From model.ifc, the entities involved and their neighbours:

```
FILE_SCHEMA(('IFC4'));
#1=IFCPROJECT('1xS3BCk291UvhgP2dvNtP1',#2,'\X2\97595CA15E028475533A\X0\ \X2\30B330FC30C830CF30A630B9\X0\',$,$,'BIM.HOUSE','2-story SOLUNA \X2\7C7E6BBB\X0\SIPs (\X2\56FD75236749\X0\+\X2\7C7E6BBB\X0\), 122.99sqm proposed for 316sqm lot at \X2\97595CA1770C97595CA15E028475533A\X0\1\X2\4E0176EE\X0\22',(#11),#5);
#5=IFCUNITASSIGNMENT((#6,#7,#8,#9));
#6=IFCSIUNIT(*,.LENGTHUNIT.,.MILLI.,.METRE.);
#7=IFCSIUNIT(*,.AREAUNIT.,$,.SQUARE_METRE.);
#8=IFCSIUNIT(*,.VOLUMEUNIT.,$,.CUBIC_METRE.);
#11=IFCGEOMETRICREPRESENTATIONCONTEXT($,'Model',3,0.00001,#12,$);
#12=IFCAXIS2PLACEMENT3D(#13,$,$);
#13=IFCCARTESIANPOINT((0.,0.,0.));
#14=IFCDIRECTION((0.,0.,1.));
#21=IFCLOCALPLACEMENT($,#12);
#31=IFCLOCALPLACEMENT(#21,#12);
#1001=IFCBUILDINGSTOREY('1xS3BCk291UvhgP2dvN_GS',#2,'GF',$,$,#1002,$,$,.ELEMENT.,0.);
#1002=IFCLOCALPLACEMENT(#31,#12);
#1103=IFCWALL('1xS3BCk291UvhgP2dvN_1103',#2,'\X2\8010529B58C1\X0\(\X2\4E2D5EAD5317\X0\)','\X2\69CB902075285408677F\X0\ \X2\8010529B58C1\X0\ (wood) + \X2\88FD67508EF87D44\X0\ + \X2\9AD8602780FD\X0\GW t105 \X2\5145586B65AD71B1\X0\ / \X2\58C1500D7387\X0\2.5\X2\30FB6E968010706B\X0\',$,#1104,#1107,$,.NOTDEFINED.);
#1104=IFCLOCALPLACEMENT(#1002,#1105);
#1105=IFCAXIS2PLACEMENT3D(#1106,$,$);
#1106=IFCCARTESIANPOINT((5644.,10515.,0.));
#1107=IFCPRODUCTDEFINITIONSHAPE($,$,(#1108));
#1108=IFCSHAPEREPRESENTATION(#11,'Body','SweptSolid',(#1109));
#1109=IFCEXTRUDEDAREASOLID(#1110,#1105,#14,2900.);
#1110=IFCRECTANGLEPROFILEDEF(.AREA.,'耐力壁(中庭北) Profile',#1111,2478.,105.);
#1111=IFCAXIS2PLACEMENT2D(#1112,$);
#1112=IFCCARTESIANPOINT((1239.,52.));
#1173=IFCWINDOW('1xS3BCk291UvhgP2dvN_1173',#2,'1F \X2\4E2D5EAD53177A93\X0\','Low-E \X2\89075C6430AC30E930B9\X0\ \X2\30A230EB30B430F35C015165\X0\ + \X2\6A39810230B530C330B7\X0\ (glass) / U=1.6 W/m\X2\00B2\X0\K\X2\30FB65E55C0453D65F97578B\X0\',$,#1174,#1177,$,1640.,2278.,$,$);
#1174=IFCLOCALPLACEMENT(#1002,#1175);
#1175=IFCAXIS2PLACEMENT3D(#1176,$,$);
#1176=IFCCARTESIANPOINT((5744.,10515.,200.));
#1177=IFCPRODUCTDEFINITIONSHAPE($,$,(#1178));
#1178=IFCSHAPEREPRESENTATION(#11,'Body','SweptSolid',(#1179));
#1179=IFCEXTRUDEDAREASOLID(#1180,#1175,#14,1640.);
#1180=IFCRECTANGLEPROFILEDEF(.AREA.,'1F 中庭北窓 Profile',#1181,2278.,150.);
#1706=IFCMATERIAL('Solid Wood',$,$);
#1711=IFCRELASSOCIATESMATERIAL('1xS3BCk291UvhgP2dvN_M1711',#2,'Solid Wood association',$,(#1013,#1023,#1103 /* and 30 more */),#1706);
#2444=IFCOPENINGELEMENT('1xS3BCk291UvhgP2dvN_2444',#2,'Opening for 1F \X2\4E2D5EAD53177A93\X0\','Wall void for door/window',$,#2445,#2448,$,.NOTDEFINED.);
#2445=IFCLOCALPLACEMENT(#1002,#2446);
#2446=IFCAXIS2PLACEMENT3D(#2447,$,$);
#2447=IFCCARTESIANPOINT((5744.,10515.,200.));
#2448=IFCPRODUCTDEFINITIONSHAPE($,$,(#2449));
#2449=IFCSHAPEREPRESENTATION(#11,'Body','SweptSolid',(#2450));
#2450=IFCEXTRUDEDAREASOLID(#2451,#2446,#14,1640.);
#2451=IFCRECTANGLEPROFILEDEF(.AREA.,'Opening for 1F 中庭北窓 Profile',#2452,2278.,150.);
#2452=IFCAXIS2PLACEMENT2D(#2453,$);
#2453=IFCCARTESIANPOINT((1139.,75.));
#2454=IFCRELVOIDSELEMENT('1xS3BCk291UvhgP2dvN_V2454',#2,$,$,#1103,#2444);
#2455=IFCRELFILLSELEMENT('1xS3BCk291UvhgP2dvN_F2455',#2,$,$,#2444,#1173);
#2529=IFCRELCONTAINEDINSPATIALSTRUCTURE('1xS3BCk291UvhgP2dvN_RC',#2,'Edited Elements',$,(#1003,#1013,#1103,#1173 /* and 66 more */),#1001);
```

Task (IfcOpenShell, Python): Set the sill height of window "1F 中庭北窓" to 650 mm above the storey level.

```python
import numpy as np
import ifcopenshell
import ifcopenshell.api.geometry
import ifcopenshell.geom
import ifcopenshell.util.element
import ifcopenshell.util.placement
import ifcopenshell.util.shape
import ifcopenshell.util.unit

model = ifcopenshell.open("model.ifc")
unit_scale = ifcopenshell.util.unit.calculate_unit_scale(model)

window = model.by_guid("1xS3BCk291UvhgP2dvN_1173")
opening = window.FillsVoids[0].RelatingOpeningElement
storey = ifcopenshell.util.element.get_container(window, ifc_class="IfcBuildingStorey")
level = ifcopenshell.util.placement.get_local_placement(storey.ObjectPlacement)[2, 3]

# The opening's origin need not be at the sill, so measure its lowest point.
shape = ifcopenshell.geom.create_shape(ifcopenshell.geom.settings(), opening)
bottom = ifcopenshell.util.shape.get_shape_bottom_elevation(shape, shape.geometry) / unit_scale
dz = level + 650.0 - bottom

shift = np.array([0.0, 0.0, dz])
# The window is not placed relative to its opening, so move both.
for product in (opening, window):
    matrix = ifcopenshell.util.placement.get_local_placement(product.ObjectPlacement)
    matrix[:3, 3] += shift
    ifcopenshell.api.geometry.edit_object_placement(model, product=product, matrix=matrix, is_si=False)

print(f"moved by {dz * unit_scale:+.3f} m")

model.write("model_rev.ifc")
```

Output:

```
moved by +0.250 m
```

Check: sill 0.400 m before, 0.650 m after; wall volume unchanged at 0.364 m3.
